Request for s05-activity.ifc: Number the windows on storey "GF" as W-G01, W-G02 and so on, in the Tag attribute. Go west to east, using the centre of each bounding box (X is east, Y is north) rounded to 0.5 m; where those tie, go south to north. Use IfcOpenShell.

First a look at what the model holds.

```python
import ifcopenshell
import ifcopenshell.util.element
import ifcopenshell.util.placement

model = ifcopenshell.open("s05-activity.ifc")
print(model.schema)
storey = next(s for s in model.by_type("IfcBuildingStorey") if s.Name == "GF")
windows = [e for e in ifcopenshell.util.element.get_decomposition(storey) if e.is_a("IfcWindow")]
for e in sorted(windows, key=lambda e: e.id()):
    origin = ifcopenshell.util.placement.get_local_placement(e.ObjectPlacement)[:3, 3]
    print(e.id(), e.Tag, e.Name, origin.round(2) + 0.0, sep=" | ")
```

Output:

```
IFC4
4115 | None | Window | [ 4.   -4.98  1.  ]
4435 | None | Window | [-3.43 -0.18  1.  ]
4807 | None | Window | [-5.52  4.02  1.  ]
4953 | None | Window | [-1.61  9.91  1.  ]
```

```python
import ifcopenshell
import ifcopenshell.geom
import ifcopenshell.util.element
import ifcopenshell.util.shape

model = ifcopenshell.open("s05-activity.ifc")
settings = ifcopenshell.geom.settings()
settings.set("use-world-coords", True)


def centre(element):
    shape = ifcopenshell.geom.create_shape(settings, element)
    return ifcopenshell.util.shape.get_bbox_centroid(shape.geometry)


storey = next(s for s in model.by_type("IfcBuildingStorey") if s.Name == "GF")
windows = [e for e in ifcopenshell.util.element.get_decomposition(storey) if e.is_a("IfcWindow")]

# Insertion points can sit at a corner or the storey origin, so sort by the geometry (in metres).
centres = {e: centre(e) for e in windows}
windows.sort(key=lambda e: (round(centres[e][0] / 0.5), centres[e][1]))

for i, e in enumerate(windows, start=1):
    number = f"W-G{i:02d}"
    e.Tag = number
    print(e.id(), number)

model.write("s05-activity_rev.ifc")
```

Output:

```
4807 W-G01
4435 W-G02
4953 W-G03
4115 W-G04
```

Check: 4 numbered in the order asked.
